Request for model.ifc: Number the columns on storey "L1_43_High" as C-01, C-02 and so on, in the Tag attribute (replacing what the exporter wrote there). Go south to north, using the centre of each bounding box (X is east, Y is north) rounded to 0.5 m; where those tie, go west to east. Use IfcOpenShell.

First a look at what the model holds.

```python
import ifcopenshell
import ifcopenshell.util.element
import ifcopenshell.util.placement

model = ifcopenshell.open("model.ifc")
print(model.schema)
storey = next(s for s in model.by_type("IfcBuildingStorey") if s.Name == "L1_43_High")
columns = [e for e in ifcopenshell.util.element.get_decomposition(storey) if e.is_a("IfcColumn")]
for e in sorted(columns, key=lambda e: e.id()):
    origin = ifcopenshell.util.placement.get_local_placement(e.ObjectPlacement)[:3, 3]
    print(e.id(), e.Tag, e.Name, origin.round(2) + 0.0, sep=" | ")
```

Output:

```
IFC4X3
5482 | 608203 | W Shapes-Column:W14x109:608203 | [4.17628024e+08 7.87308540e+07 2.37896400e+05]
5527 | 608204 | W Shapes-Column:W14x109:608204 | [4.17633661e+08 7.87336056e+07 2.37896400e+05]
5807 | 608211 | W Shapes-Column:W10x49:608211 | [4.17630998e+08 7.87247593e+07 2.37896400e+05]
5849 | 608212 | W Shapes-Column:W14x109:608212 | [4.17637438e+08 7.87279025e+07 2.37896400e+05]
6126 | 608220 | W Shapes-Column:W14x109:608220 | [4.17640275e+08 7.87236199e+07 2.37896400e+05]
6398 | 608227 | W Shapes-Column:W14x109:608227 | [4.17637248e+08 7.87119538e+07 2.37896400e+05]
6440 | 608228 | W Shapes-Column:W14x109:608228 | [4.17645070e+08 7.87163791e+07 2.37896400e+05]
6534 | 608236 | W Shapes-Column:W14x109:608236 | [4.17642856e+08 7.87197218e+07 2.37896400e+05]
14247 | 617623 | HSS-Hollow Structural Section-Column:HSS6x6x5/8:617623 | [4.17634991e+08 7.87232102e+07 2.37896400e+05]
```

```python
import ifcopenshell
import ifcopenshell.geom
import ifcopenshell.util.element
import ifcopenshell.util.shape

model = ifcopenshell.open("model.ifc")
settings = ifcopenshell.geom.settings()
settings.set("use-world-coords", True)


def centre(element):
    shape = ifcopenshell.geom.create_shape(settings, element)
    return ifcopenshell.util.shape.get_bbox_centroid(shape.geometry)


storey = next(s for s in model.by_type("IfcBuildingStorey") if s.Name == "L1_43_High")
columns = [e for e in ifcopenshell.util.element.get_decomposition(storey) if e.is_a("IfcColumn")]

# Insertion points can sit at a corner or the storey origin, so sort by the geometry (in metres).
centres = {e: centre(e) for e in columns}
columns.sort(key=lambda e: (round(centres[e][1] / 0.5), centres[e][0]))

for i, e in enumerate(columns, start=1):
    number = f"C-{i:02d}"
    e.Tag = number
    print(e.id(), number)

model.write("model_edited.ifc")
```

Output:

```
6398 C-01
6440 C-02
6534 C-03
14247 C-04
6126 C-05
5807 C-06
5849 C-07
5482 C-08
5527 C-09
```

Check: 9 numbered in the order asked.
